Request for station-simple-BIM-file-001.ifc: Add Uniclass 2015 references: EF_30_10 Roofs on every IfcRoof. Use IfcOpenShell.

First a look at what the model holds.

```python
import ifcopenshell

model = ifcopenshell.open("station-simple-BIM-file-001.ifc")
print(model.schema)
print("classifications:", [c.Name for c in model.by_type("IfcClassification")])
for ifc_class in ("IfcDoor", "IfcRoof", "IfcStair", "IfcWall", "IfcWindow"):
    print(ifc_class, len(model.by_type(ifc_class)))
```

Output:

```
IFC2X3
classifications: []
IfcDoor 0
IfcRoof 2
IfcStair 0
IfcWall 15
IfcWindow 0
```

```python
import ifcopenshell
import ifcopenshell.api.classification

model = ifcopenshell.open("station-simple-BIM-file-001.ifc")

# IFC2X3 requires Source and Edition and has no link from the project to the system.
system = model.create_entity("IfcClassification", Source="NBS", Edition="2015", Name="Uniclass 2015")

codes = {
    "IfcRoof": ("EF_30_10", "Roofs"),
}
for ifc_class, (code, name) in codes.items():
    products = model.by_type(ifc_class)
    ifcopenshell.api.classification.add_reference(
        model, products=products, classification=system, identification=code, name=name
    )
    print(code, len(products))

model.write("station-simple-BIM-file-001-out.ifc")
```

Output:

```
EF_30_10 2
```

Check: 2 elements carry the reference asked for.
